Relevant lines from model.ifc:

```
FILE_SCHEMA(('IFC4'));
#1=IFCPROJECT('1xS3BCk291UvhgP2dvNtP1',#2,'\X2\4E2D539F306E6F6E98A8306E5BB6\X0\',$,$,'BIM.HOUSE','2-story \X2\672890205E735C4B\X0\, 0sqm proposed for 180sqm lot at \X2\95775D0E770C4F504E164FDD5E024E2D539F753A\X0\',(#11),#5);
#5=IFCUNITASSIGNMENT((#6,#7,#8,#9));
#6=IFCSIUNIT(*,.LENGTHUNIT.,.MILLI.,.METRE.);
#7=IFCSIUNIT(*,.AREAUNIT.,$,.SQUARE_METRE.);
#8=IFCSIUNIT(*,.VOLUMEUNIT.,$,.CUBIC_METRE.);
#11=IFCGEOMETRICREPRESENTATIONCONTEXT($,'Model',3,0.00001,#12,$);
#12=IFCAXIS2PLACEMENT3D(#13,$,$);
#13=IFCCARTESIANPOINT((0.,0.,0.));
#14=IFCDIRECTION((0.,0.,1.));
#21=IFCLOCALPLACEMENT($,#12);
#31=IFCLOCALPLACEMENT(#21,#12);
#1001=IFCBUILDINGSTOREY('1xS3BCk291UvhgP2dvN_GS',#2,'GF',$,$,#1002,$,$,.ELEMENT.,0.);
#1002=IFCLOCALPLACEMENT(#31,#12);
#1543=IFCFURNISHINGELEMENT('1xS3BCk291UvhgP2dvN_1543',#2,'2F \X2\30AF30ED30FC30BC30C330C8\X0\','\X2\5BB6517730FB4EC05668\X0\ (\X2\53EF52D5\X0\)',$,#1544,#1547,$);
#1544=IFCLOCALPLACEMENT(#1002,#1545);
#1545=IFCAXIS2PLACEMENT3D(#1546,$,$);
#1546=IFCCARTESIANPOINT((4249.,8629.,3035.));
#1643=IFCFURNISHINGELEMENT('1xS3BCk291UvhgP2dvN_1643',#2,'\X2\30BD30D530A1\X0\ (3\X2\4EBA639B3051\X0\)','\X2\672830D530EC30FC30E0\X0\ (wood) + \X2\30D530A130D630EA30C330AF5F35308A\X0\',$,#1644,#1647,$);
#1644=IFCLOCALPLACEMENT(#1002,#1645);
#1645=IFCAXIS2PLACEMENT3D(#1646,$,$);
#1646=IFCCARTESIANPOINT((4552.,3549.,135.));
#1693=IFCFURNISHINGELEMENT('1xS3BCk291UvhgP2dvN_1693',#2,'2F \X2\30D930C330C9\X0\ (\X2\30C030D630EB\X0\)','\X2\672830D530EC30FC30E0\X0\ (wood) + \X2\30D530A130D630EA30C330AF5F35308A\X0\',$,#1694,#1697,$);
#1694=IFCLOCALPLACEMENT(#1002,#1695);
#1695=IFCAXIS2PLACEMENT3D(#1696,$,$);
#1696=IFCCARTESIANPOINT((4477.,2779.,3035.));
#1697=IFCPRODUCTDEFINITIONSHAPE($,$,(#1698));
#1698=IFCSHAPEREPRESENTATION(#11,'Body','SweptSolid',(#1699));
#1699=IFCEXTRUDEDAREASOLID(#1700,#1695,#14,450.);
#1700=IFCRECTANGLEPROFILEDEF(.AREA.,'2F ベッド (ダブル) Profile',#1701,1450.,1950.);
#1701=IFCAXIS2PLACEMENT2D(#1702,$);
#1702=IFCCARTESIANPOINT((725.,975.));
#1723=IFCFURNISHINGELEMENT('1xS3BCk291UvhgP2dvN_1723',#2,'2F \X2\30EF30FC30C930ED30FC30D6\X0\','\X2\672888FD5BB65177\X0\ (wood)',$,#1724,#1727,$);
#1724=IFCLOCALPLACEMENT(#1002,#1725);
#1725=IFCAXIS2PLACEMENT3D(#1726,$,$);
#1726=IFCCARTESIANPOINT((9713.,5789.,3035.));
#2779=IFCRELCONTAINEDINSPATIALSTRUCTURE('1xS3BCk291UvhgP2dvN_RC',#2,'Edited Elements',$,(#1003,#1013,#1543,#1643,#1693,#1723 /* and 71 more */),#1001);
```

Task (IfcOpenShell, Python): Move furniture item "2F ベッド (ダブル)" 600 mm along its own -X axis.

```python
import ifcopenshell
import ifcopenshell.api.geometry
import ifcopenshell.util.placement

model = ifcopenshell.open("model.ifc")

item = model.by_guid("1xS3BCk291UvhgP2dvN_1693")
matrix = ifcopenshell.util.placement.get_local_placement(item.ObjectPlacement)
matrix[:3, 3] -= matrix[:3, 0] * 600.0
ifcopenshell.api.geometry.edit_object_placement(model, product=item, matrix=matrix, is_si=False)

print(ifcopenshell.util.placement.get_local_placement(item.ObjectPlacement).round(3) + 0.0)

model.write("model-out.ifc")
```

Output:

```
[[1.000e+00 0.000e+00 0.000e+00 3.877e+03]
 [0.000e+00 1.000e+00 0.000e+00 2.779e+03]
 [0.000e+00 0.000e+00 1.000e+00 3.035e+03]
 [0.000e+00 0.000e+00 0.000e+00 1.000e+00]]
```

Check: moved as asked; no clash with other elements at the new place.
